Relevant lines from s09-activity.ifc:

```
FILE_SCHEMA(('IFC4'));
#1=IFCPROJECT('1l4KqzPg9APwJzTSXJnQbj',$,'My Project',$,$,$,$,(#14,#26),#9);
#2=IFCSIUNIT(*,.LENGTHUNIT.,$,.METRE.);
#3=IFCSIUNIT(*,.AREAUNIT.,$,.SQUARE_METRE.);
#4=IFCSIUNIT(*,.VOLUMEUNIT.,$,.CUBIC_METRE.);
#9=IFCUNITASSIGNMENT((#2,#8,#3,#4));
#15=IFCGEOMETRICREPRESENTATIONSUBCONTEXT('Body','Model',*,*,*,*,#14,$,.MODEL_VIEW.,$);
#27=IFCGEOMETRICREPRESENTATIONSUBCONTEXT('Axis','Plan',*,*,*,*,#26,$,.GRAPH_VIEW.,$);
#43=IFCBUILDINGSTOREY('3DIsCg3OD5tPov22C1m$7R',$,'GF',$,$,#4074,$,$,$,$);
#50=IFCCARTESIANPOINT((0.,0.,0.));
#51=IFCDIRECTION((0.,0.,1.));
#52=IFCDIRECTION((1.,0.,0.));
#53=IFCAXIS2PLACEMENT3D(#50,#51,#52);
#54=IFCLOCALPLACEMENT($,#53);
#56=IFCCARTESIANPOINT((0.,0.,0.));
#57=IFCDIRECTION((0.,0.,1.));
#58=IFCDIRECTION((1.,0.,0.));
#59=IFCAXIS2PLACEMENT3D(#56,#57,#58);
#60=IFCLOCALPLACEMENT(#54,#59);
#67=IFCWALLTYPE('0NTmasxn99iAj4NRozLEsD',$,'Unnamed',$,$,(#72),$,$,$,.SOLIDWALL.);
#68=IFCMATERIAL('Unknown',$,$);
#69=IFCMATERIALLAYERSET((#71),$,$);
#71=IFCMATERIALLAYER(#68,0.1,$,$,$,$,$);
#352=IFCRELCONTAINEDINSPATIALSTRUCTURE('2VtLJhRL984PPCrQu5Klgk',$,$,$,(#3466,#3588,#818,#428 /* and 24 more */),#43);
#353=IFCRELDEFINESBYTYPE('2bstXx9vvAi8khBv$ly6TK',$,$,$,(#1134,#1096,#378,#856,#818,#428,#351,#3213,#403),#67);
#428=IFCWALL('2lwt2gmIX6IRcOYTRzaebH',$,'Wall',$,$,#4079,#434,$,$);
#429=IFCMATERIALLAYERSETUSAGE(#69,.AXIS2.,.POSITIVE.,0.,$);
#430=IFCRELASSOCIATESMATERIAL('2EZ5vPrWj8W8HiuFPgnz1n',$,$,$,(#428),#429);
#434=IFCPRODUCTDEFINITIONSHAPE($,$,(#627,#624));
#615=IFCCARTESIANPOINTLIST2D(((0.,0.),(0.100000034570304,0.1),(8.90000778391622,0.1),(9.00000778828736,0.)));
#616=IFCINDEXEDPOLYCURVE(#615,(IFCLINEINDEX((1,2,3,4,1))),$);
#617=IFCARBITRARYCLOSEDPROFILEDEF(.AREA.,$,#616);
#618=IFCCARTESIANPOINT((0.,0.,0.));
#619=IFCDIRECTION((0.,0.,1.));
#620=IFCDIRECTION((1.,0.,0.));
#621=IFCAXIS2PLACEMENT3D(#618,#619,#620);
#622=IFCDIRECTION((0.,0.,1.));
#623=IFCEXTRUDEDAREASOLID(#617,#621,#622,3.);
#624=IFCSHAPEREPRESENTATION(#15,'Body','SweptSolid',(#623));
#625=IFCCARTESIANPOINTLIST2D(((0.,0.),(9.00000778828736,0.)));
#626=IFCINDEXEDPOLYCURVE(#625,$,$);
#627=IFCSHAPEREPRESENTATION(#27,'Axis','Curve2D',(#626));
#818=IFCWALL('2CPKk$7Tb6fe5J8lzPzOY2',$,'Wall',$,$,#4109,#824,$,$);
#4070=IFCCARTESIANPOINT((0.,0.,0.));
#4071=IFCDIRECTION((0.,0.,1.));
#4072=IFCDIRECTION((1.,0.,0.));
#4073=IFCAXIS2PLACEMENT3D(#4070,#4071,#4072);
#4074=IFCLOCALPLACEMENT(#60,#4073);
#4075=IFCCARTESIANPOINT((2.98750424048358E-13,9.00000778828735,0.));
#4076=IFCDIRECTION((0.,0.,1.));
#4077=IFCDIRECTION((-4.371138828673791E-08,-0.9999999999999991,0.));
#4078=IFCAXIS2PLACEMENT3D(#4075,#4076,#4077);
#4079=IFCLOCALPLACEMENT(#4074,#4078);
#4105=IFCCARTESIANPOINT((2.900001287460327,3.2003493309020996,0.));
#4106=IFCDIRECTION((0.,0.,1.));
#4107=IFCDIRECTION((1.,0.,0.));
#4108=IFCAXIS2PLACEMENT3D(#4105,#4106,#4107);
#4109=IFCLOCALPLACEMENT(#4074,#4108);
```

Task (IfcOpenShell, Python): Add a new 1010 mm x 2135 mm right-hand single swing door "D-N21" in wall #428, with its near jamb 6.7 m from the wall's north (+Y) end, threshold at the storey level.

```python
import numpy as np
import ifcopenshell
import ifcopenshell.api.feature
import ifcopenshell.api.geometry
import ifcopenshell.api.root
import ifcopenshell.api.spatial
import ifcopenshell.geom
import ifcopenshell.util.element
import ifcopenshell.util.placement
import ifcopenshell.util.representation
import ifcopenshell.util.shape
import ifcopenshell.util.unit

model = ifcopenshell.open("s09-activity.ifc")
unit_scale = ifcopenshell.util.unit.calculate_unit_scale(model)
settings = ifcopenshell.geom.settings()


def volume(element):
    """Net volume in cubic metres, openings subtracted."""
    shape = ifcopenshell.geom.create_shape(settings, element)
    return ifcopenshell.util.shape.get_volume(shape.geometry)


wall = model.by_guid("2lwt2gmIX6IRcOYTRzaebH")
storey = ifcopenshell.util.element.get_container(wall, ifc_class="IfcBuildingStorey")
context = ifcopenshell.util.representation.get_context(model, "Model", "Body", "MODEL_VIEW")
before = volume(wall)

width, height, from_end, sill = 1.01, 2.135, 6.7, 0.0  # metres

# The wall runs along its own X axis, and the end named is its -X end.
wall_shape = ifcopenshell.geom.create_shape(settings, wall)
x, y, z = ifcopenshell.util.shape.get_vertices(wall_shape.geometry).T
start = x.min() + from_end
face, thickness = float(y.min()), float(y.max() - y.min())
wall_matrix = ifcopenshell.util.placement.get_local_placement(wall.ObjectPlacement)
level = ifcopenshell.util.placement.get_local_placement(storey.ObjectPlacement)[2, 3]


def in_wall(x, y):
    """Placement at x, y metres in the wall's axes, at sill height."""
    matrix = wall_matrix.copy()
    matrix[:, 3] = wall_matrix @ np.array([x / unit_scale, y / unit_scale, 0.0, 1.0])
    matrix[2, 3] = level + sill / unit_scale
    return matrix


# Opening: a box that overshoots both wall faces by 50 mm.
opening = ifcopenshell.api.root.create_entity(model, ifc_class="IfcOpeningElement", predefined_type="OPENING")
box = ifcopenshell.api.geometry.add_wall_representation(
    model, context=context, length=width, height=height, thickness=thickness + 0.1
)
ifcopenshell.api.geometry.assign_representation(model, product=opening, representation=box)
ifcopenshell.api.geometry.edit_object_placement(model, product=opening, matrix=in_wall(start, face - 0.05), is_si=False)
ifcopenshell.api.feature.add_feature(model, feature=opening, element=wall)

door = ifcopenshell.api.root.create_entity(model, ifc_class="IfcDoor", name="D-N21", predefined_type="DOOR")
door.OverallWidth, door.OverallHeight = width / unit_scale, height / unit_scale
door.OperationType = "SINGLE_SWING_RIGHT"
body = ifcopenshell.api.geometry.add_door_representation(
    model,
    context=context,
    overall_width=door.OverallWidth,
    overall_height=door.OverallHeight,
    operation_type="SINGLE_SWING_RIGHT",
    lining_properties={"LiningDepth": thickness / unit_scale, "ThresholdDepth": thickness / unit_scale},
)
ifcopenshell.api.geometry.assign_representation(model, product=door, representation=body)
ifcopenshell.api.spatial.assign_container(model, products=[door], relating_structure=storey)
ifcopenshell.api.feature.add_filling(model, opening=opening, element=door)

# The lining spans the wall, so the door starts at the wall face.
ifcopenshell.api.geometry.edit_object_placement(model, product=door, matrix=in_wall(start, face), is_si=False)

after = volume(wall)

print(f"wall volume {before:.3f} -> {after:.3f} m3")

model.write("s09-activity-out.ifc")
```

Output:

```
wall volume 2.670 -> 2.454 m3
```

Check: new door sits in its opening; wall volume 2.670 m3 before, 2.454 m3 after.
